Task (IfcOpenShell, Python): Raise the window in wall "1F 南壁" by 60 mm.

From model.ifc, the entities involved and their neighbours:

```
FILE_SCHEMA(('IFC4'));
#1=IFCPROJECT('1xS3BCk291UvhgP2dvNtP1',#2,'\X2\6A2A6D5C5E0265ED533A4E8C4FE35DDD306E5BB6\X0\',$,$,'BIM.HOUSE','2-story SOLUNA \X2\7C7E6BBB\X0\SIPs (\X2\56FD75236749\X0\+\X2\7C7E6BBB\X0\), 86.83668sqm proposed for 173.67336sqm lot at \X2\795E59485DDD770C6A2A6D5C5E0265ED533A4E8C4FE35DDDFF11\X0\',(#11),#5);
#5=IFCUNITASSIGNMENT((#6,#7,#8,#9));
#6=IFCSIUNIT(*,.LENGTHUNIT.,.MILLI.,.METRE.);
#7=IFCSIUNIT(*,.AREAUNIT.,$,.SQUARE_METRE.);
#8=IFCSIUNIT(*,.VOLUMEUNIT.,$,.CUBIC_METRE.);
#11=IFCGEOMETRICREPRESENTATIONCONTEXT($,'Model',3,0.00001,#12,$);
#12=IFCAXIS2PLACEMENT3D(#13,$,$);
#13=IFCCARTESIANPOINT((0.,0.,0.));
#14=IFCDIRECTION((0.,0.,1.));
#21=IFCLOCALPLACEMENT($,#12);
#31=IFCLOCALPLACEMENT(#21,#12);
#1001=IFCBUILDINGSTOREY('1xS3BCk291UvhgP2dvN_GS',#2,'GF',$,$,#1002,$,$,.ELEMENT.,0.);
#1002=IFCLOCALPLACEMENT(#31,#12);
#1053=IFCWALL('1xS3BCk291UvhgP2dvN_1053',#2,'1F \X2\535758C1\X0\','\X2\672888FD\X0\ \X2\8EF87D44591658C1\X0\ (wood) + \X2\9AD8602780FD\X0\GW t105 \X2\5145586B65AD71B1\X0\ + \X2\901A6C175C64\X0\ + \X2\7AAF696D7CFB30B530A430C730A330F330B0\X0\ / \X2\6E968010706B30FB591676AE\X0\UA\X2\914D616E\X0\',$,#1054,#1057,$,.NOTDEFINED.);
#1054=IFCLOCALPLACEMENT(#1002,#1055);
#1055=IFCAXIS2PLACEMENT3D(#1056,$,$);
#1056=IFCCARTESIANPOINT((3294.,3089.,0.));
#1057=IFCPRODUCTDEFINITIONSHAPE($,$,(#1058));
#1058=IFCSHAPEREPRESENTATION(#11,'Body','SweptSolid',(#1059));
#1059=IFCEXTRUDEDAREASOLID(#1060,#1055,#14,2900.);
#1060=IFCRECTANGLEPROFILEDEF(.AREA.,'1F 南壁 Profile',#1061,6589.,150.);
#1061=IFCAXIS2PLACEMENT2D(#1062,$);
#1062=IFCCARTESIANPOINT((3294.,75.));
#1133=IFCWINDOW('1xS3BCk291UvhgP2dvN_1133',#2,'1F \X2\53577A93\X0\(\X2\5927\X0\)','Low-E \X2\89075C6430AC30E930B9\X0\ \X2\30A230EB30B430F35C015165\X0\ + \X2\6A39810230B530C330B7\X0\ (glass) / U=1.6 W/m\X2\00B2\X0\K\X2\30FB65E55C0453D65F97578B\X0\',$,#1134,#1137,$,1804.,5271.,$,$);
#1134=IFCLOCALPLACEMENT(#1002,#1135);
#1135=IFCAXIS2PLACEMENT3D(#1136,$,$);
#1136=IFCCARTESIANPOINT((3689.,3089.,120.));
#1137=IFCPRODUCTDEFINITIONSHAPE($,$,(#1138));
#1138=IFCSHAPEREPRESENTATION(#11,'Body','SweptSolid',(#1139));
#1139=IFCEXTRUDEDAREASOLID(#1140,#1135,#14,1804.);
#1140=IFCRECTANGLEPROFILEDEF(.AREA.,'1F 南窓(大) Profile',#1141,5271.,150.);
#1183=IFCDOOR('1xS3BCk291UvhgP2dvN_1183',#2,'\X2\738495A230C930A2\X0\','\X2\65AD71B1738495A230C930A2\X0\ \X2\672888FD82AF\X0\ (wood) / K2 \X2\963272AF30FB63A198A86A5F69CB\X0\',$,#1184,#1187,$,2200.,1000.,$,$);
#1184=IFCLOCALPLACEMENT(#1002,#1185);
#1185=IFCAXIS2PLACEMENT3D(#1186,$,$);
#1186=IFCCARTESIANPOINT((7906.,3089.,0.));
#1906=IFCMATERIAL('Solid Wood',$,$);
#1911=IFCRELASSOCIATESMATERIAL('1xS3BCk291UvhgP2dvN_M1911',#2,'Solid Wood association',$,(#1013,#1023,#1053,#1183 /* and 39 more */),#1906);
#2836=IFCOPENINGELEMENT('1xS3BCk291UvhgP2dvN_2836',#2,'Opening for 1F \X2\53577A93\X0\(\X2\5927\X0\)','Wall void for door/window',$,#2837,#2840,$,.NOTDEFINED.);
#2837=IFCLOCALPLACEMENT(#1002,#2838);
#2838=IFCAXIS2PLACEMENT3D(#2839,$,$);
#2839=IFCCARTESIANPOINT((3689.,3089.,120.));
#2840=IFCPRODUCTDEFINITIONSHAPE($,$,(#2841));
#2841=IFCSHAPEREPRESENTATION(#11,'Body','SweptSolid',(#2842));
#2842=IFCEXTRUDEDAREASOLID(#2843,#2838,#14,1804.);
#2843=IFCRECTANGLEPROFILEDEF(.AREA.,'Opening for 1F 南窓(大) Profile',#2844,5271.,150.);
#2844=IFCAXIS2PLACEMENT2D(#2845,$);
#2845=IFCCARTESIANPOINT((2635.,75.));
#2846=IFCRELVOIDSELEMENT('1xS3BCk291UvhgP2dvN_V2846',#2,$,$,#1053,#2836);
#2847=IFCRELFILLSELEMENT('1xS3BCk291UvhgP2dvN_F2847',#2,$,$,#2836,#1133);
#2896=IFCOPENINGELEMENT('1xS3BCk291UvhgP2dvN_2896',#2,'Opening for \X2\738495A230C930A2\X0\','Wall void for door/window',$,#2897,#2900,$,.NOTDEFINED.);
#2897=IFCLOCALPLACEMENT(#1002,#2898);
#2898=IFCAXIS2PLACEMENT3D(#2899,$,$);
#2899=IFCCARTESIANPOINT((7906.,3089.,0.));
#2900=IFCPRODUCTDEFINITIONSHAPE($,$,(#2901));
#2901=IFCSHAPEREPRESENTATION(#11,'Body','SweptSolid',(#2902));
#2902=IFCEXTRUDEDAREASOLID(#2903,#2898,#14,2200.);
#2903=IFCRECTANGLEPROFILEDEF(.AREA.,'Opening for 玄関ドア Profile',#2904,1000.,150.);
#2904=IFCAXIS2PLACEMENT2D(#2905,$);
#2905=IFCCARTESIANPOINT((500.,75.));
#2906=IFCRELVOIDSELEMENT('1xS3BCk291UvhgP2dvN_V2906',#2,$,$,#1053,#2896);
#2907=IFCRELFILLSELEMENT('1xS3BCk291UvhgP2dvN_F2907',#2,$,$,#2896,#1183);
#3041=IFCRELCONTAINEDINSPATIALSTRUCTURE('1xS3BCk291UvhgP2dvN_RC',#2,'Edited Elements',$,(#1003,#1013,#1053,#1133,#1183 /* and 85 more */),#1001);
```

```python
import numpy as np
import ifcopenshell
import ifcopenshell.api.geometry
import ifcopenshell.util.placement
import ifcopenshell.util.unit

model = ifcopenshell.open("model.ifc")
unit_scale = ifcopenshell.util.unit.calculate_unit_scale(model)

window = model.by_guid("1xS3BCk291UvhgP2dvN_1133")
opening = window.FillsVoids[0].RelatingOpeningElement
dz = 60.0

shift = np.array([0.0, 0.0, dz])
# The window is not placed relative to its opening, so move both.
for product in (opening, window):
    matrix = ifcopenshell.util.placement.get_local_placement(product.ObjectPlacement)
    matrix[:3, 3] += shift
    ifcopenshell.api.geometry.edit_object_placement(model, product=product, matrix=matrix, is_si=False)

print(f"moved by {dz * unit_scale:+.3f} m")

model.write("model_edited.ifc")
```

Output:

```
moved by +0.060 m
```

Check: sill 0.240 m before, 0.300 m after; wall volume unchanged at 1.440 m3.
